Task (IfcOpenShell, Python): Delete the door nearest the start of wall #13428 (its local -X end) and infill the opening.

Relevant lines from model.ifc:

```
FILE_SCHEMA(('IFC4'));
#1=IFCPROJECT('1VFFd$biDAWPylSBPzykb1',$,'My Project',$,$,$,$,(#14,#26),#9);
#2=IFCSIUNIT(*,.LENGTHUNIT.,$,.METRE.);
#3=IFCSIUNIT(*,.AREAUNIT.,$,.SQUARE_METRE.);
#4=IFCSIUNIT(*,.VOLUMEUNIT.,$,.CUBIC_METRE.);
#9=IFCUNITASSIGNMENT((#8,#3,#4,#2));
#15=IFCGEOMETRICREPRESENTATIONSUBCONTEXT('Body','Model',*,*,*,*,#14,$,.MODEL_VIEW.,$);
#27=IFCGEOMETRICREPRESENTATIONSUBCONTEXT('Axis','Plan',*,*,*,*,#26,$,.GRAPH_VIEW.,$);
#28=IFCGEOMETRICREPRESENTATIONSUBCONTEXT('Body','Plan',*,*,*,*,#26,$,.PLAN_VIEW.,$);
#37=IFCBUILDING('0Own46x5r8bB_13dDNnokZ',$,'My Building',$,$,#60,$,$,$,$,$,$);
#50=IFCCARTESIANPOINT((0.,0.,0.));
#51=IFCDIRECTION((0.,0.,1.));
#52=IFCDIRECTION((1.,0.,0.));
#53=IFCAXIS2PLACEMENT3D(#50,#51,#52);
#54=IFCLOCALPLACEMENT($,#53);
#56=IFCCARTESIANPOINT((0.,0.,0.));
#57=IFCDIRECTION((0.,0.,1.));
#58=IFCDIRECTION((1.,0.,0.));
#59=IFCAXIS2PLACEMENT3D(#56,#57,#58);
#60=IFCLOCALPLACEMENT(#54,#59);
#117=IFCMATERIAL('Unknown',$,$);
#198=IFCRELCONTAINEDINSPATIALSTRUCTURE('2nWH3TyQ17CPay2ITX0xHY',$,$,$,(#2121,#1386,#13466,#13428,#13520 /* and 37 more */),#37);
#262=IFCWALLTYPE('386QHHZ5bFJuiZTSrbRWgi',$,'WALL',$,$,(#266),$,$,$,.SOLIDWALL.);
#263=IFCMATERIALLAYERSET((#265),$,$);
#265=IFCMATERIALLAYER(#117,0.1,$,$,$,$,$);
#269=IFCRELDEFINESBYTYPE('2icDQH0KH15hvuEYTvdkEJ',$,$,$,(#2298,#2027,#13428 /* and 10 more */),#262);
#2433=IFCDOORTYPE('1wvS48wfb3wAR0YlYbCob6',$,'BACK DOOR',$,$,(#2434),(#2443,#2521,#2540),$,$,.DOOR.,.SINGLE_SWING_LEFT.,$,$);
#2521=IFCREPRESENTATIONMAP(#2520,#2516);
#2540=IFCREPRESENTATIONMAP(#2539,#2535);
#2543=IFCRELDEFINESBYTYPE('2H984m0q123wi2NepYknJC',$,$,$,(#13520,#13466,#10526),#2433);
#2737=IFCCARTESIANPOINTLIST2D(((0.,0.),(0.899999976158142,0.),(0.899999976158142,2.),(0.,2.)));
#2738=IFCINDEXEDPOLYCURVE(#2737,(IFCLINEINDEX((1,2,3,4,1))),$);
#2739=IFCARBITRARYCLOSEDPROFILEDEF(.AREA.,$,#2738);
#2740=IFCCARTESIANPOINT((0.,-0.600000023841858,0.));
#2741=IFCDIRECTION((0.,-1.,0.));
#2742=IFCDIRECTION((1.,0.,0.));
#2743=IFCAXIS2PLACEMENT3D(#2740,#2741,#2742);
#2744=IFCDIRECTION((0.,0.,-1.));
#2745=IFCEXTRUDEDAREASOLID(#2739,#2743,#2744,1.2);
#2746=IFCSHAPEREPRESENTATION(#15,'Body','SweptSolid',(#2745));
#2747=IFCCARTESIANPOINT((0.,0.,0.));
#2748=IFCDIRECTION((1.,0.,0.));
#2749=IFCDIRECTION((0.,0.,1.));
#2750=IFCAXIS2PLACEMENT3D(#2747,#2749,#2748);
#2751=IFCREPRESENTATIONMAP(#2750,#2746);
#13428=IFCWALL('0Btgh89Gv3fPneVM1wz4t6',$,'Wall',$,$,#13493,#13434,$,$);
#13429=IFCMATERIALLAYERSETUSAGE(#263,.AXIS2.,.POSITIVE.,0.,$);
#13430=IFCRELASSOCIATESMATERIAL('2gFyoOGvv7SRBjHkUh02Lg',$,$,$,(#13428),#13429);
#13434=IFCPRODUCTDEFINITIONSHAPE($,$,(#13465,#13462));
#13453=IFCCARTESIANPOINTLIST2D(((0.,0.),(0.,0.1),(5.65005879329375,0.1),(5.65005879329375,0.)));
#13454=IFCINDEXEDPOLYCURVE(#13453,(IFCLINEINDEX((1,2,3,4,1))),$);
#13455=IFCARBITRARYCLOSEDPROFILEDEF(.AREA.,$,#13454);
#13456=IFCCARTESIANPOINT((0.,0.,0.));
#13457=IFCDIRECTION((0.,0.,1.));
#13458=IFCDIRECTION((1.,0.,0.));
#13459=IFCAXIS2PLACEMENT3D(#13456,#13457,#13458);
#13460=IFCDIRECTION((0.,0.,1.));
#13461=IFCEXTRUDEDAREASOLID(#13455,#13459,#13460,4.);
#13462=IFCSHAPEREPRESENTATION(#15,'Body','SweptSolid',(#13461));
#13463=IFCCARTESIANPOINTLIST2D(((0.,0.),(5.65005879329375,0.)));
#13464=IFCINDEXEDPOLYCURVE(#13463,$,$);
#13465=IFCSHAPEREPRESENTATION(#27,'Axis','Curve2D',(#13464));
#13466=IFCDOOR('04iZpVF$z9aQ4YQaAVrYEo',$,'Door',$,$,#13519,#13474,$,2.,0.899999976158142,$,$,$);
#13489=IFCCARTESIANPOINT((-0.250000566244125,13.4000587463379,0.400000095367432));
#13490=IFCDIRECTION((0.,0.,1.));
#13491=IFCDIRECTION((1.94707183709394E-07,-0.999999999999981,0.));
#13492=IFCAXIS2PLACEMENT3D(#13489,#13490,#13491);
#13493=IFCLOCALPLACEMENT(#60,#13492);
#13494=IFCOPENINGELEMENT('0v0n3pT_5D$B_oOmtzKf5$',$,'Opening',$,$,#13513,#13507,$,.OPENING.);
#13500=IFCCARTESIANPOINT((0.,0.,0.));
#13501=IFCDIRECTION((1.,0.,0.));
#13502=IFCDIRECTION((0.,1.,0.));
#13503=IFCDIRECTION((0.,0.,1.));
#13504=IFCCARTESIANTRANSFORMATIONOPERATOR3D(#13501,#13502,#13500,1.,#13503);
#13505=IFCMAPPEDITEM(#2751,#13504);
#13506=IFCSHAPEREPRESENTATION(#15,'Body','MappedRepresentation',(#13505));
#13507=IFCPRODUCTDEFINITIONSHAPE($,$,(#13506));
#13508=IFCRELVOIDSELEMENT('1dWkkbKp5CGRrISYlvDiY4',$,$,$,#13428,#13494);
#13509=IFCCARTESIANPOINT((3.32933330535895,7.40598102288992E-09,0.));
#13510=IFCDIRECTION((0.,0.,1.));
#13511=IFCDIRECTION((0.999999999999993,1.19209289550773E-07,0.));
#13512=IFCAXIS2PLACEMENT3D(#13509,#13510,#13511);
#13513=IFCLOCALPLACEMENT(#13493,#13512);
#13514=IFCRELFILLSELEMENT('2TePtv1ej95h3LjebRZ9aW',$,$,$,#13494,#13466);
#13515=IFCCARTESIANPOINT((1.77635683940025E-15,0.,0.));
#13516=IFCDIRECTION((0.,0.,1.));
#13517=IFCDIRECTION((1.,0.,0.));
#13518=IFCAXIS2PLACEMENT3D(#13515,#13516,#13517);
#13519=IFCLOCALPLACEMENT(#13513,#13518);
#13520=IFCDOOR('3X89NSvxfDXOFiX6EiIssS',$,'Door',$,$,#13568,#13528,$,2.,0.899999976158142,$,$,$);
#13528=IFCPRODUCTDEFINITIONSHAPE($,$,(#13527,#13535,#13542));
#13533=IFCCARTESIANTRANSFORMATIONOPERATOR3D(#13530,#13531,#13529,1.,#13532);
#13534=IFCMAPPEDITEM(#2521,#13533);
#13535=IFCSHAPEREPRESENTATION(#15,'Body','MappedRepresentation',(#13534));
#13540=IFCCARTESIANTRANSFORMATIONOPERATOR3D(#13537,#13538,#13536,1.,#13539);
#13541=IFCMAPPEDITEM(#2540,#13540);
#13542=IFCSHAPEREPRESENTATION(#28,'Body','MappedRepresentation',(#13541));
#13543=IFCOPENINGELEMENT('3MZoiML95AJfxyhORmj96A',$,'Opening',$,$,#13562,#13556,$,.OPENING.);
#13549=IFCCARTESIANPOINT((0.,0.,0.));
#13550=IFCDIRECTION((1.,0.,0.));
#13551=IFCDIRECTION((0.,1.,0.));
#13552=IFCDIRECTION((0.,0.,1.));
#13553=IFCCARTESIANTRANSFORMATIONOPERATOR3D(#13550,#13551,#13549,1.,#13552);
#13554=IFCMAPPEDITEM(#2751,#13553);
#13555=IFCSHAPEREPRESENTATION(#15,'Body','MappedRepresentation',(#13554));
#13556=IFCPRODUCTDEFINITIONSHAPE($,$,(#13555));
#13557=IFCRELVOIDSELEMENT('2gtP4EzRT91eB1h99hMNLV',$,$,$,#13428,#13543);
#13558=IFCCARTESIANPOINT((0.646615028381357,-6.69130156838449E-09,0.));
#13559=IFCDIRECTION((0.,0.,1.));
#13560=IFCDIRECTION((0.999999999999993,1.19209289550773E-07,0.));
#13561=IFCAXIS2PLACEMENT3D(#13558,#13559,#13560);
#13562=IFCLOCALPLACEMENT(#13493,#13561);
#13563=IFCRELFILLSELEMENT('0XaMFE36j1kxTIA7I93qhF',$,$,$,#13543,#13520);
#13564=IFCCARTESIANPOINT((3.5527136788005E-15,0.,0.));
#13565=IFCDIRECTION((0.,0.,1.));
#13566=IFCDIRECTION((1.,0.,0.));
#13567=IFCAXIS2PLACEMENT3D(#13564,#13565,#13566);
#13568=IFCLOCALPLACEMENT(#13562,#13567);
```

```python
import ifcopenshell
import ifcopenshell.api.feature
import ifcopenshell.api.root
import ifcopenshell.geom
import ifcopenshell.util.shape

model = ifcopenshell.open("model.ifc")
settings = ifcopenshell.geom.settings()


def volume(element):
    """Net volume in cubic metres, openings subtracted."""
    shape = ifcopenshell.geom.create_shape(settings, element)
    return ifcopenshell.util.shape.get_volume(shape.geometry)


door = model.by_id(13520)
opening = door.FillsVoids[0].RelatingOpeningElement
wall = opening.VoidsElements[0].RelatingBuildingElement
before = volume(wall)

ifcopenshell.api.root.remove_product(model, product=door)
ifcopenshell.api.feature.remove_feature(model, feature=opening)

after = volume(wall)

print(f"wall volume {before:.3f} -> {after:.3f} m3")

model.write("model_edited.ifc")
```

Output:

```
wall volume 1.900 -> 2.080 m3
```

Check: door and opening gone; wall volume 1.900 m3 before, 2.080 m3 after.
